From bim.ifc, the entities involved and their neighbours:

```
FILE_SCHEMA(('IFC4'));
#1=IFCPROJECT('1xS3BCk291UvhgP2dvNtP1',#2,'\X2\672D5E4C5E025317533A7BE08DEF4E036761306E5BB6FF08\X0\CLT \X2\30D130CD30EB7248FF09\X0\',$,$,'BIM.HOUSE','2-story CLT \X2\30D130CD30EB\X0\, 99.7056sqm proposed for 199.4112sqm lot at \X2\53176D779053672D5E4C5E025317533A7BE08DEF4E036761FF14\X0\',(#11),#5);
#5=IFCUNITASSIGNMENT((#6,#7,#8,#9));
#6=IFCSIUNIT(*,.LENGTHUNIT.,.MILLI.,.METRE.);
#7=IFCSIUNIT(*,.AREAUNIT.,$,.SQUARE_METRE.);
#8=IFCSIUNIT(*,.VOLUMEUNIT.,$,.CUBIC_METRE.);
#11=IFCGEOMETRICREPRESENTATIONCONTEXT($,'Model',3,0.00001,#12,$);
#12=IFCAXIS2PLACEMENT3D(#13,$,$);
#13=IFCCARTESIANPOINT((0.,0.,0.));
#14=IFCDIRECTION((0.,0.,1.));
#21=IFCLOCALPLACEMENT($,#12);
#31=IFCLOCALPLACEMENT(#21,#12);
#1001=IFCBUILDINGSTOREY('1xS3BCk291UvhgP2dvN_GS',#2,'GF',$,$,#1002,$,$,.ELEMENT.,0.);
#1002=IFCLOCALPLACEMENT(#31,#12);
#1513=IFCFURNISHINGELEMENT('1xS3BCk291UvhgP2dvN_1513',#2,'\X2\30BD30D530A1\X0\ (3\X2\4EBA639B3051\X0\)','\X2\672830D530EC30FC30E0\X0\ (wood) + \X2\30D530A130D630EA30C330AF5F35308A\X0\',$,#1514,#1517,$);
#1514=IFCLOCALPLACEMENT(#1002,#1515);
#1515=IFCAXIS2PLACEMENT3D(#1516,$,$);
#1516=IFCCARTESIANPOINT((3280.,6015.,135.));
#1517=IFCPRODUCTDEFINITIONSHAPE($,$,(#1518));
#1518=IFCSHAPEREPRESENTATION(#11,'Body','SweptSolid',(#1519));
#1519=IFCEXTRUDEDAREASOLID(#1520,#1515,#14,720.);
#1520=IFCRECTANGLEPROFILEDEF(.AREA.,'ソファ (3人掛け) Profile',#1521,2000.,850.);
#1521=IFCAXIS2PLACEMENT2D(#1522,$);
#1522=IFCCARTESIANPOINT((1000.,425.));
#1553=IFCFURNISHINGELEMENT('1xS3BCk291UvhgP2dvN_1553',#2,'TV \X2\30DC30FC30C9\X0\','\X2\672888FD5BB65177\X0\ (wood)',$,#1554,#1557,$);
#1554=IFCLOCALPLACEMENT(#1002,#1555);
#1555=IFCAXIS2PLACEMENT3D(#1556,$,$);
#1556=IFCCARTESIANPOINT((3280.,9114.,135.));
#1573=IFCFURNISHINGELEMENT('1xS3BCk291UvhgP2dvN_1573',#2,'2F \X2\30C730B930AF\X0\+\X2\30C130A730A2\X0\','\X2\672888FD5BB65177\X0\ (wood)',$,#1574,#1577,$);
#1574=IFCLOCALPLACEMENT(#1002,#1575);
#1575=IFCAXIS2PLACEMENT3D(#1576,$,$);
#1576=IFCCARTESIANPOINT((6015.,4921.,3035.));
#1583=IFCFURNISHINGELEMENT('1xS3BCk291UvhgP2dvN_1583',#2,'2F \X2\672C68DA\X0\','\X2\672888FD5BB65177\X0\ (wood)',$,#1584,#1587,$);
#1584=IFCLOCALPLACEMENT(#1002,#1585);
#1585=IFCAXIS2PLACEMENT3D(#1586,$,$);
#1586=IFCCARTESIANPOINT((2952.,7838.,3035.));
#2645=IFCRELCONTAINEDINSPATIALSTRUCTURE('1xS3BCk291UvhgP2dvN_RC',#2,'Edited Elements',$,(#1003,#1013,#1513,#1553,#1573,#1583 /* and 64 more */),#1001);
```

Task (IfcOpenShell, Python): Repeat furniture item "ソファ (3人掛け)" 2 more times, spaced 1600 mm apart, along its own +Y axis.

```python
import ifcopenshell
import ifcopenshell.api.geometry
import ifcopenshell.api.root
import ifcopenshell.util.element
import ifcopenshell.util.placement

model = ifcopenshell.open("bim.ifc")


def reuse_history(source, copy):
    """copy_class also copies each property set's owner history, people and application; keep the originals."""
    for rel in copy.IsDefinedBy:
        if rel.is_a("IfcRelDefinesByProperties") and (history := rel.RelatingPropertyDefinition.OwnerHistory):
            rel.RelatingPropertyDefinition.OwnerHistory = source.OwnerHistory
            ifcopenshell.util.element.remove_deep2(model, history)


source = model.by_id(1513)
base = ifcopenshell.util.placement.get_local_placement(source.ObjectPlacement)
step = base[:3, 1] * 1600.0

for i in range(1, 3):
    copy = ifcopenshell.api.root.copy_class(model, product=source)
    copy.Representation = ifcopenshell.util.element.copy_deep(
        model, source.Representation, exclude=["IfcGeometricRepresentationContext", "IfcRepresentationMap"]
    )
    reuse_history(source, copy)
    matrix = base.copy()
    matrix[:3, 3] += i * step
    print("added at", matrix[:3, 3].round(3) + 0.0)
    ifcopenshell.api.geometry.edit_object_placement(model, product=copy, matrix=matrix, is_si=False)

model.write("bim_edited.ifc")
```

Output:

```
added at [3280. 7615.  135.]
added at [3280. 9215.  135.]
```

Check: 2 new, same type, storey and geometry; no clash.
